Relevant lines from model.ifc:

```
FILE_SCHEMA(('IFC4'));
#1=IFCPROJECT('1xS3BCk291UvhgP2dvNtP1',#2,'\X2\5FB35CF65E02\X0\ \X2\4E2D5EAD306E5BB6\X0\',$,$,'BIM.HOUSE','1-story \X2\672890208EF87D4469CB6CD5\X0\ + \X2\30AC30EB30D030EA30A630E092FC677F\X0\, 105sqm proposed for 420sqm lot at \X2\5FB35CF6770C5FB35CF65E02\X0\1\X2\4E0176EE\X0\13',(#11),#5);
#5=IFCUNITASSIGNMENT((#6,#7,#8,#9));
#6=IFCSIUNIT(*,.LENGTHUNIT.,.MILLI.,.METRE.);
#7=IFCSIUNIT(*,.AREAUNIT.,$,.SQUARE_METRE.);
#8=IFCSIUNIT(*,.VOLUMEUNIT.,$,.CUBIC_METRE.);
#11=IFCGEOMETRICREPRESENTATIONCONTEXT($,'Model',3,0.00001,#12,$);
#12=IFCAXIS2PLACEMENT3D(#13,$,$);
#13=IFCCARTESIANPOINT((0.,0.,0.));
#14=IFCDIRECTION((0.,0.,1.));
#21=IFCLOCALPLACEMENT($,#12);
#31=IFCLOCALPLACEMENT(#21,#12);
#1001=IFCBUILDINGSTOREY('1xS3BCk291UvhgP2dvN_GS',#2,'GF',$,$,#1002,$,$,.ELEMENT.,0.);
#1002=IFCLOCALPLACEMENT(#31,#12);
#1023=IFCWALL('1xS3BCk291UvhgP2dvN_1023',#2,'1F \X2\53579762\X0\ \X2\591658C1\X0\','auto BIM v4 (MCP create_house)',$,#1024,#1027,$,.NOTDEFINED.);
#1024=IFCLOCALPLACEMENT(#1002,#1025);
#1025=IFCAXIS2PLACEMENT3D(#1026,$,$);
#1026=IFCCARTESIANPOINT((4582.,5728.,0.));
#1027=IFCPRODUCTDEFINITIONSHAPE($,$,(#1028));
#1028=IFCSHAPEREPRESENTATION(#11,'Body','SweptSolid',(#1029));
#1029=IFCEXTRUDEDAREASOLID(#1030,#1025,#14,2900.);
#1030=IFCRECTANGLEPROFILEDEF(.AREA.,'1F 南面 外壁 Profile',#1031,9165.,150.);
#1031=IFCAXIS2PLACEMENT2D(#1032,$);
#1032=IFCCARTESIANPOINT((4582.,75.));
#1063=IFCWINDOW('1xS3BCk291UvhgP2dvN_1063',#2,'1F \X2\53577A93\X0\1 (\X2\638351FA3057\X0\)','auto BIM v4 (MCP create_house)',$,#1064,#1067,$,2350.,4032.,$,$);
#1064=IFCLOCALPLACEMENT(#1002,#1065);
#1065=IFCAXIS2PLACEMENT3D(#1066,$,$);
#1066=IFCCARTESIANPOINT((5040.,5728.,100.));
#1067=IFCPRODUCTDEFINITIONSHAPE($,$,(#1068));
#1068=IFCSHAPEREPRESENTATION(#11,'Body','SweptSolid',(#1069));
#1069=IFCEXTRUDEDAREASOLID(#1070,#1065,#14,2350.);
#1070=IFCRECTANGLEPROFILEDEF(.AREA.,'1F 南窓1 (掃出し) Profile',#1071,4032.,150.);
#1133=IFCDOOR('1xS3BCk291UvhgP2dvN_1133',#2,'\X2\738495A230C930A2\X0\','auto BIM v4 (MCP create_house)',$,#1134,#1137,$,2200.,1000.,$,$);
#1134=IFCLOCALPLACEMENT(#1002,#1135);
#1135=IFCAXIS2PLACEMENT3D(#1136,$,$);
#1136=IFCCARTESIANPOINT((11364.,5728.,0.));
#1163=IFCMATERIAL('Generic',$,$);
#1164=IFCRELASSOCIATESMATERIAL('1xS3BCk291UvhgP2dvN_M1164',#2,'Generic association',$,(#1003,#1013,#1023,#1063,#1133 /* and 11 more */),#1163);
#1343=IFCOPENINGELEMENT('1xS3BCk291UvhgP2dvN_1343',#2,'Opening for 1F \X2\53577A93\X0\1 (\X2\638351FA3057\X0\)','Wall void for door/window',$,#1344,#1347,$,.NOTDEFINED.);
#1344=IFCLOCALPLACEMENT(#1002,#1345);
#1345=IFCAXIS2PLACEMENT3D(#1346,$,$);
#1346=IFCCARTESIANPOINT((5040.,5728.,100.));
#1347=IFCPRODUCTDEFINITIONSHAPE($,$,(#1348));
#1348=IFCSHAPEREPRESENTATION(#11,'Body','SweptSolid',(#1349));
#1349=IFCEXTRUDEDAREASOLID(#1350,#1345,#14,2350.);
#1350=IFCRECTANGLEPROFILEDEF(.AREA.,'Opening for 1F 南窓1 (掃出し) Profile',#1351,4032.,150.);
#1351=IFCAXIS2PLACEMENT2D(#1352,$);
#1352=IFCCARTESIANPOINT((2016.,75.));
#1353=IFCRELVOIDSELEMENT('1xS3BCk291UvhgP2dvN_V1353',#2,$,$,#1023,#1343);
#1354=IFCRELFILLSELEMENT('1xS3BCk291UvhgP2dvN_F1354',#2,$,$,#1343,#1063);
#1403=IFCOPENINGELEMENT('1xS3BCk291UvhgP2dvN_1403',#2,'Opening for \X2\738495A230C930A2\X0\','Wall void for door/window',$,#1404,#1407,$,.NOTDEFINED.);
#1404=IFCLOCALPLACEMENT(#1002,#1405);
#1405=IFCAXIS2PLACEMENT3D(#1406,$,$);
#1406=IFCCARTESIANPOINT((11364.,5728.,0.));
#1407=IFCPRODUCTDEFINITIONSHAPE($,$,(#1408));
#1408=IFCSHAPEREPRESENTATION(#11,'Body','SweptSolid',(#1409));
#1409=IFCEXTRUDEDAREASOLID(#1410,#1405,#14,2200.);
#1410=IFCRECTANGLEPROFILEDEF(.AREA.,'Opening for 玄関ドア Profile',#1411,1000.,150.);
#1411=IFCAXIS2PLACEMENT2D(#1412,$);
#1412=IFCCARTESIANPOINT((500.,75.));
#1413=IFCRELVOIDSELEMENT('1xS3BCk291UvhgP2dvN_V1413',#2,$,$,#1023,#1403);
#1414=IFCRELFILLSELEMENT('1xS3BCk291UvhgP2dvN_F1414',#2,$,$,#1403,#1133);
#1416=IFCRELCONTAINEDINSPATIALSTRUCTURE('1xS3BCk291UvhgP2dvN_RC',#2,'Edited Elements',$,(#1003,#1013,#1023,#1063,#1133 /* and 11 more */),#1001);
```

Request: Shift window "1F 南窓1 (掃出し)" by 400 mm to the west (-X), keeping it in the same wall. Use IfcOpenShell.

```python
import ifcopenshell
import ifcopenshell.api.geometry
import ifcopenshell.util.placement
import ifcopenshell.util.unit

model = ifcopenshell.open("model.ifc")
unit_scale = ifcopenshell.util.unit.calculate_unit_scale(model)

window = model.by_guid("1xS3BCk291UvhgP2dvN_1063")
opening = window.FillsVoids[0].RelatingOpeningElement
wall = opening.VoidsElements[0].RelatingBuildingElement

wall_matrix = ifcopenshell.util.placement.get_local_placement(wall.ObjectPlacement)
shift = wall_matrix[:3, 0] * -0.4 / unit_scale
before = ifcopenshell.util.placement.get_local_placement(window.ObjectPlacement)[:3, 3].copy()

# The window is not placed relative to its opening, so move both.
for product in (opening, window):
    matrix = ifcopenshell.util.placement.get_local_placement(product.ObjectPlacement)
    matrix[:3, 3] += shift
    ifcopenshell.api.geometry.edit_object_placement(model, product=product, matrix=matrix, is_si=False)

after = ifcopenshell.util.placement.get_local_placement(window.ObjectPlacement)[:3, 3]
print("window moved by", (after - before).round(3) + 0.0)

model.write("model_edited.ifc")
```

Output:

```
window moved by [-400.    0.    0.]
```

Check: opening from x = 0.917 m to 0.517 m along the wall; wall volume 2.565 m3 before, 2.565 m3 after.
